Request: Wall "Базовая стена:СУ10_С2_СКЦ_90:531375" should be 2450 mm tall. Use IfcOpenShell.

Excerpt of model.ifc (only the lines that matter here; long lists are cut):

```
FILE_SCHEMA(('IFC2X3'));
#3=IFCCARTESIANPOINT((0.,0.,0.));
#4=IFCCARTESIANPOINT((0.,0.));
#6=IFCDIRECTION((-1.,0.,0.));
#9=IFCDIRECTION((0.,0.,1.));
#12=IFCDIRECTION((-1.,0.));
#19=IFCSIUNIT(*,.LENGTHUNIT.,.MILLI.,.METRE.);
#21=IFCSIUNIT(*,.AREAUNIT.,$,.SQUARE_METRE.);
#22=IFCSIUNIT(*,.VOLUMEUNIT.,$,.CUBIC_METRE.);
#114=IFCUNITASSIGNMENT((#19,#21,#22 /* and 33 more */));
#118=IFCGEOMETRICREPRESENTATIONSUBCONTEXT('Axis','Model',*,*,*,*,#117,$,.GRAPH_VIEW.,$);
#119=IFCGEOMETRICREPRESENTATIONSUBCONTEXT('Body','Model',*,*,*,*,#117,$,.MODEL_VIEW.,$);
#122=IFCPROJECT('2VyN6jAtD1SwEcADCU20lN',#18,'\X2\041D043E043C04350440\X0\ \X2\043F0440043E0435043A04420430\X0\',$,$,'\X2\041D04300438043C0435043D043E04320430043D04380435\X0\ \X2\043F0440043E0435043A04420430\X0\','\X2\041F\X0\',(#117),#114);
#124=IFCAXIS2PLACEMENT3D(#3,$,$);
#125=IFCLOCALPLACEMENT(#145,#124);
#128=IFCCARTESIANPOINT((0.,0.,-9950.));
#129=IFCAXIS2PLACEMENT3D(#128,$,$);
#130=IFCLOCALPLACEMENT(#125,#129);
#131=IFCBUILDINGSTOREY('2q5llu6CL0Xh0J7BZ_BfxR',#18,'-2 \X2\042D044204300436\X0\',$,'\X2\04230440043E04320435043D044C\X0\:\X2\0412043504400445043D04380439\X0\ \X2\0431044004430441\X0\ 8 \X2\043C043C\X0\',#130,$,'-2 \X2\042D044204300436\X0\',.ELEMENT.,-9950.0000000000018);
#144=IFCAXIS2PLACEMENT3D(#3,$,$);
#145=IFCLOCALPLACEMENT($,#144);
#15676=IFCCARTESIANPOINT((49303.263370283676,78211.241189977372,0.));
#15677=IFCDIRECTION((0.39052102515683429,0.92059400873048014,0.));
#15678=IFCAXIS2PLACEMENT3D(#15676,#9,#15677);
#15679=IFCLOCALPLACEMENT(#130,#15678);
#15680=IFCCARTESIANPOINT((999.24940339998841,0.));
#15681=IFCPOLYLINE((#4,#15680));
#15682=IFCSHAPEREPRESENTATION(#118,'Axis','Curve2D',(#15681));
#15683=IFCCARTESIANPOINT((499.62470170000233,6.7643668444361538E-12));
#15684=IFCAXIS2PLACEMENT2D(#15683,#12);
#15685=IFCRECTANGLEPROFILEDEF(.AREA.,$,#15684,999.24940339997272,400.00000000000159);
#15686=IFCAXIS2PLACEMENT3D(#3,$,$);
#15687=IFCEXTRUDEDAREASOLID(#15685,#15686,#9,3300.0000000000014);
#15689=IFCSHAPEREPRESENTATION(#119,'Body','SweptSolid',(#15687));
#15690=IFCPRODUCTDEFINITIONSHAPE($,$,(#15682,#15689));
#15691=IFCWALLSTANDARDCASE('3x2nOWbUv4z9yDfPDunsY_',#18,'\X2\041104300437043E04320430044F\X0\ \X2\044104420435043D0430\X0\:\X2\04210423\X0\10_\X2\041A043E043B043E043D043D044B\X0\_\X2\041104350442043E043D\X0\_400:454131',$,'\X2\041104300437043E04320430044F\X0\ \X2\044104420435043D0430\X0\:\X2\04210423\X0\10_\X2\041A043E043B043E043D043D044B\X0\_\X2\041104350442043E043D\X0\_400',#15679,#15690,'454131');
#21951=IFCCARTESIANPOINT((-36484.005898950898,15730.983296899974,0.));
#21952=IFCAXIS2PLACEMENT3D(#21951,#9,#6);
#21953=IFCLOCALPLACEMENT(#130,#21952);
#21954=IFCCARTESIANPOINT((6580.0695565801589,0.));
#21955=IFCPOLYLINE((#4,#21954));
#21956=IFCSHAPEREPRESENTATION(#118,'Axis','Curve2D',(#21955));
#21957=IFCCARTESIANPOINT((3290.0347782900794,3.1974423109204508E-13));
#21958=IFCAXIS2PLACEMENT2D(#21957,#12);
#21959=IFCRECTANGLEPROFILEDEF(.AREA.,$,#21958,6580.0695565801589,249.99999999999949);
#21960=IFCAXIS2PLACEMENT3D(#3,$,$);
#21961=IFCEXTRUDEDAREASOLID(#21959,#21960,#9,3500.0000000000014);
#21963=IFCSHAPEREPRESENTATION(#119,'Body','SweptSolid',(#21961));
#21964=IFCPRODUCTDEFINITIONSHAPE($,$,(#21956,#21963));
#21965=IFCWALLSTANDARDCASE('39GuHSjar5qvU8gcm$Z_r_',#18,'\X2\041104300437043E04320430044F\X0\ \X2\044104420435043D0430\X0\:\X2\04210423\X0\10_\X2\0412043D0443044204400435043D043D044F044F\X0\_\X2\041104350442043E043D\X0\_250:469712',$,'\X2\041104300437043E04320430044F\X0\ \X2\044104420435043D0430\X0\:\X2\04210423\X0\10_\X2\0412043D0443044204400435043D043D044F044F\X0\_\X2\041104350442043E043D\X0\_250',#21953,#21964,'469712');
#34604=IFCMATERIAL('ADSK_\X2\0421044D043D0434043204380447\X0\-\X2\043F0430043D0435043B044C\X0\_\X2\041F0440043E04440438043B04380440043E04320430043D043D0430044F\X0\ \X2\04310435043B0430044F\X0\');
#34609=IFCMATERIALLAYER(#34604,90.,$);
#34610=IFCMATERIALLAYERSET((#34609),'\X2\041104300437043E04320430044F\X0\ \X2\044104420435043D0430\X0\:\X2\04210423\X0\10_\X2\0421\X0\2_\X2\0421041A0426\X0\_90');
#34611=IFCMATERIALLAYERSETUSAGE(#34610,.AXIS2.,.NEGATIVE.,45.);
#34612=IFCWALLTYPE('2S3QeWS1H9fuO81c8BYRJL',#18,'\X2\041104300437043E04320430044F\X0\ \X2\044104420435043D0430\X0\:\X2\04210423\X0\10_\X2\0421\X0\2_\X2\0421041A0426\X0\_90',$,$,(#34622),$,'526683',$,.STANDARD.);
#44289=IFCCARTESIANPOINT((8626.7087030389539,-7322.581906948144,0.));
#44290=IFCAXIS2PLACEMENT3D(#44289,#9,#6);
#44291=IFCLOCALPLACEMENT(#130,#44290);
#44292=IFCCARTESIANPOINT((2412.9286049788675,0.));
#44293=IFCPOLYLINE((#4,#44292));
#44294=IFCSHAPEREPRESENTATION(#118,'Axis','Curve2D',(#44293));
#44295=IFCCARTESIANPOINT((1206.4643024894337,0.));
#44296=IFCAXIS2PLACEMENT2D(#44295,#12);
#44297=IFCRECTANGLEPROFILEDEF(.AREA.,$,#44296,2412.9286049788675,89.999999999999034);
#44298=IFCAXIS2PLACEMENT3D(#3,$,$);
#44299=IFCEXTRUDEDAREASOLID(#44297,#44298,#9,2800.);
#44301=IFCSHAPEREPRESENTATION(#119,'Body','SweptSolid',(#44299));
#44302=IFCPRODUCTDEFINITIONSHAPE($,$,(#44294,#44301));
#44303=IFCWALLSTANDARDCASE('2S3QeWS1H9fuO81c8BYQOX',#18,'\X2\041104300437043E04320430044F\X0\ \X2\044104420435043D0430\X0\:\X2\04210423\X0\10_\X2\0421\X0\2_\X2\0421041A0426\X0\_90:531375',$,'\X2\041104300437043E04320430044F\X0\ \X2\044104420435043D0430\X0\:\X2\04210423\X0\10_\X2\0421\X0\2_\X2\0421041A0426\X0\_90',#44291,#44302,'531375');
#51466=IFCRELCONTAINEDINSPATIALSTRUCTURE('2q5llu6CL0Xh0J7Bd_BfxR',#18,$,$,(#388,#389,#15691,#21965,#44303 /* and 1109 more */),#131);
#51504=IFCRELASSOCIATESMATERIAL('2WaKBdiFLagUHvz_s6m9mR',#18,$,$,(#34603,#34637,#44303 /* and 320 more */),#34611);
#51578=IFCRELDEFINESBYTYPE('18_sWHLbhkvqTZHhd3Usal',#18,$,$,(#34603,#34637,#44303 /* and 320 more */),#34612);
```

```python
import ifcopenshell
import ifcopenshell.geom
import ifcopenshell.util.representation
import ifcopenshell.util.shape
import ifcopenshell.util.unit

model = ifcopenshell.open("model.ifc")
unit_scale = ifcopenshell.util.unit.calculate_unit_scale(model)
settings = ifcopenshell.geom.settings()


def volume(element):
    """Net volume in cubic metres, openings subtracted."""
    shape = ifcopenshell.geom.create_shape(settings, element)
    return ifcopenshell.util.shape.get_volume(shape.geometry)


wall = model.by_id(44303)
before = volume(wall)

body = ifcopenshell.util.representation.get_representation(wall, "Model", "Body")
solid = body.Items[0]
old_height = solid.Depth
solid.Depth = 2.45 / unit_scale
after = volume(wall)

print(f"height {old_height:g} -> {solid.Depth:g}, volume {before:.3f} -> {after:.3f} m3")

model.write("model_updated.ifc")
```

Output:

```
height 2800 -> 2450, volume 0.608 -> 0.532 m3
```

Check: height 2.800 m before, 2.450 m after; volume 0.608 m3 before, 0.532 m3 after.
